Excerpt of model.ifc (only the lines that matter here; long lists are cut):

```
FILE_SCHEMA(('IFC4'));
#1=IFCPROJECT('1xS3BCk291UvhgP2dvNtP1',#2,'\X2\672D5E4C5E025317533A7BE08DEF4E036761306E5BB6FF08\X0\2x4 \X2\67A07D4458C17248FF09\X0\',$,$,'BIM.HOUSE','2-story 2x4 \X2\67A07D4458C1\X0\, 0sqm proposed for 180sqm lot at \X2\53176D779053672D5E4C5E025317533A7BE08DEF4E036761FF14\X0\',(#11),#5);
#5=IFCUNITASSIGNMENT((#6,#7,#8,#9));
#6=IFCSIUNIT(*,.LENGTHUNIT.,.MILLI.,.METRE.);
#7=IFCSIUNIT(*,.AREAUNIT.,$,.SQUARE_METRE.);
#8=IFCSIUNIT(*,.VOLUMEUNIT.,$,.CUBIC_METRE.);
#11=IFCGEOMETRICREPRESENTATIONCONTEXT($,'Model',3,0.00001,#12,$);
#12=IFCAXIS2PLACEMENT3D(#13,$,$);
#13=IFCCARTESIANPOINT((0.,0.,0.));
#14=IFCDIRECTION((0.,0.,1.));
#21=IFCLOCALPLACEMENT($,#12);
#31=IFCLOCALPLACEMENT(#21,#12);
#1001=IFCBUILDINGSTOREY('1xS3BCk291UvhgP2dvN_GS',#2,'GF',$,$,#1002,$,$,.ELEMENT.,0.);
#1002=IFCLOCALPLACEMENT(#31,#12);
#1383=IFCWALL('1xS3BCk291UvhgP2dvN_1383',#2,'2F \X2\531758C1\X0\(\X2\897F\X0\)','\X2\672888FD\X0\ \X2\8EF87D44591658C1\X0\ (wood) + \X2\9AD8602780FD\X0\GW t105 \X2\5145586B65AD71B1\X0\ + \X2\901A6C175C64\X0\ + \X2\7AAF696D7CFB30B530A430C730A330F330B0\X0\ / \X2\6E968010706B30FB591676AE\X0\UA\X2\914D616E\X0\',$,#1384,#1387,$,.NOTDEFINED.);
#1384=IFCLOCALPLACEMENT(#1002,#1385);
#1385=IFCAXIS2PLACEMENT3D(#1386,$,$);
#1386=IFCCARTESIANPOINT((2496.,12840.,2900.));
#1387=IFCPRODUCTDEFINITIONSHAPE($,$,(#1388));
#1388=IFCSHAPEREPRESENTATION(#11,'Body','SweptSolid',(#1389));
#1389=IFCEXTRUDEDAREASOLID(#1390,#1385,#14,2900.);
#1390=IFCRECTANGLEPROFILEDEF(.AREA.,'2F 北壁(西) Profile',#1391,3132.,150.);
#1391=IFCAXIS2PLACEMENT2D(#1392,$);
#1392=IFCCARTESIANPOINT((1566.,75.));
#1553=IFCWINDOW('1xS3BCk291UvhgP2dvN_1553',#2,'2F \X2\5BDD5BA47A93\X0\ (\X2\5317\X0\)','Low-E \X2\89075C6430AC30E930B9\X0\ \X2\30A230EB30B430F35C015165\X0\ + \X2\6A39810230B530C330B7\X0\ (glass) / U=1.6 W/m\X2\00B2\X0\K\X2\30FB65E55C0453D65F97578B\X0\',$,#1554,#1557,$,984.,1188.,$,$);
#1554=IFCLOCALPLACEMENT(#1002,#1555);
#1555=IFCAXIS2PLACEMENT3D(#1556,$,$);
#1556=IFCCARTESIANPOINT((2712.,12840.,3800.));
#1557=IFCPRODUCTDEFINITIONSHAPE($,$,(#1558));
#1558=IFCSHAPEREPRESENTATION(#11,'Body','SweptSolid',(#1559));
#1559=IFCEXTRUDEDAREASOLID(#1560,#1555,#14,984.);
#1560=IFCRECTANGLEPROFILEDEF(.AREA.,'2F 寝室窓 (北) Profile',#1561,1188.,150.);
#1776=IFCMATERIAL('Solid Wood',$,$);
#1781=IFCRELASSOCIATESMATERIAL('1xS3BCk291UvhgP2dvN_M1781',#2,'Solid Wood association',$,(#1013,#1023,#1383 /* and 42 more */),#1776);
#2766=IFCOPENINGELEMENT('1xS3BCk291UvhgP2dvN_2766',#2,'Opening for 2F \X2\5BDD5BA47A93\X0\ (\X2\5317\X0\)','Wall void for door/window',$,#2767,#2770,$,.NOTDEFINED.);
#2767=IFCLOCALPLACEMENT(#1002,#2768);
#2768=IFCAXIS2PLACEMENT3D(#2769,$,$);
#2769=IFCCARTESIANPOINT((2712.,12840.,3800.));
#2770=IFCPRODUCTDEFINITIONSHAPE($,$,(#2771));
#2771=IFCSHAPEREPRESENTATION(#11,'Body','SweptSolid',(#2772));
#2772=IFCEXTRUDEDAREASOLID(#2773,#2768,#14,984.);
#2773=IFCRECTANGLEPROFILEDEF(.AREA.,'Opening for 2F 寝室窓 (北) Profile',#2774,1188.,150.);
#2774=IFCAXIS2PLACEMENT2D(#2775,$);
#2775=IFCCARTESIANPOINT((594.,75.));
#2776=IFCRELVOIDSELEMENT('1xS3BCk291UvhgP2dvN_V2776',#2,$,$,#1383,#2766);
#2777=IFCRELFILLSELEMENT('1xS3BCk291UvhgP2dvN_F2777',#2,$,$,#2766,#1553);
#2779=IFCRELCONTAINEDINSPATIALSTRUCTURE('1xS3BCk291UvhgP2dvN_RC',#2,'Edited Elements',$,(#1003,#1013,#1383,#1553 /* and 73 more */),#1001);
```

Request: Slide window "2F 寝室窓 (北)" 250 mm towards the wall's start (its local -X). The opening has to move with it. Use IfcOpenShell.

```python
import ifcopenshell
import ifcopenshell.api.geometry
import ifcopenshell.util.placement
import ifcopenshell.util.unit

model = ifcopenshell.open("model.ifc")
unit_scale = ifcopenshell.util.unit.calculate_unit_scale(model)

window = model.by_id(1553)
opening = window.FillsVoids[0].RelatingOpeningElement
wall = opening.VoidsElements[0].RelatingBuildingElement

wall_matrix = ifcopenshell.util.placement.get_local_placement(wall.ObjectPlacement)
shift = wall_matrix[:3, 0] * -0.25 / unit_scale
before = ifcopenshell.util.placement.get_local_placement(window.ObjectPlacement)[:3, 3].copy()

# The window is not placed relative to its opening, so move both.
for product in (opening, window):
    matrix = ifcopenshell.util.placement.get_local_placement(product.ObjectPlacement)
    matrix[:3, 3] += shift
    ifcopenshell.api.geometry.edit_object_placement(model, product=product, matrix=matrix, is_si=False)

after = ifcopenshell.util.placement.get_local_placement(window.ObjectPlacement)[:3, 3]
print("window moved by", (after - before).round(3) + 0.0)

model.write("model_v2.ifc")
```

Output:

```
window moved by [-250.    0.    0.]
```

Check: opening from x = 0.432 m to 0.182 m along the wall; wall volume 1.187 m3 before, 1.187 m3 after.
